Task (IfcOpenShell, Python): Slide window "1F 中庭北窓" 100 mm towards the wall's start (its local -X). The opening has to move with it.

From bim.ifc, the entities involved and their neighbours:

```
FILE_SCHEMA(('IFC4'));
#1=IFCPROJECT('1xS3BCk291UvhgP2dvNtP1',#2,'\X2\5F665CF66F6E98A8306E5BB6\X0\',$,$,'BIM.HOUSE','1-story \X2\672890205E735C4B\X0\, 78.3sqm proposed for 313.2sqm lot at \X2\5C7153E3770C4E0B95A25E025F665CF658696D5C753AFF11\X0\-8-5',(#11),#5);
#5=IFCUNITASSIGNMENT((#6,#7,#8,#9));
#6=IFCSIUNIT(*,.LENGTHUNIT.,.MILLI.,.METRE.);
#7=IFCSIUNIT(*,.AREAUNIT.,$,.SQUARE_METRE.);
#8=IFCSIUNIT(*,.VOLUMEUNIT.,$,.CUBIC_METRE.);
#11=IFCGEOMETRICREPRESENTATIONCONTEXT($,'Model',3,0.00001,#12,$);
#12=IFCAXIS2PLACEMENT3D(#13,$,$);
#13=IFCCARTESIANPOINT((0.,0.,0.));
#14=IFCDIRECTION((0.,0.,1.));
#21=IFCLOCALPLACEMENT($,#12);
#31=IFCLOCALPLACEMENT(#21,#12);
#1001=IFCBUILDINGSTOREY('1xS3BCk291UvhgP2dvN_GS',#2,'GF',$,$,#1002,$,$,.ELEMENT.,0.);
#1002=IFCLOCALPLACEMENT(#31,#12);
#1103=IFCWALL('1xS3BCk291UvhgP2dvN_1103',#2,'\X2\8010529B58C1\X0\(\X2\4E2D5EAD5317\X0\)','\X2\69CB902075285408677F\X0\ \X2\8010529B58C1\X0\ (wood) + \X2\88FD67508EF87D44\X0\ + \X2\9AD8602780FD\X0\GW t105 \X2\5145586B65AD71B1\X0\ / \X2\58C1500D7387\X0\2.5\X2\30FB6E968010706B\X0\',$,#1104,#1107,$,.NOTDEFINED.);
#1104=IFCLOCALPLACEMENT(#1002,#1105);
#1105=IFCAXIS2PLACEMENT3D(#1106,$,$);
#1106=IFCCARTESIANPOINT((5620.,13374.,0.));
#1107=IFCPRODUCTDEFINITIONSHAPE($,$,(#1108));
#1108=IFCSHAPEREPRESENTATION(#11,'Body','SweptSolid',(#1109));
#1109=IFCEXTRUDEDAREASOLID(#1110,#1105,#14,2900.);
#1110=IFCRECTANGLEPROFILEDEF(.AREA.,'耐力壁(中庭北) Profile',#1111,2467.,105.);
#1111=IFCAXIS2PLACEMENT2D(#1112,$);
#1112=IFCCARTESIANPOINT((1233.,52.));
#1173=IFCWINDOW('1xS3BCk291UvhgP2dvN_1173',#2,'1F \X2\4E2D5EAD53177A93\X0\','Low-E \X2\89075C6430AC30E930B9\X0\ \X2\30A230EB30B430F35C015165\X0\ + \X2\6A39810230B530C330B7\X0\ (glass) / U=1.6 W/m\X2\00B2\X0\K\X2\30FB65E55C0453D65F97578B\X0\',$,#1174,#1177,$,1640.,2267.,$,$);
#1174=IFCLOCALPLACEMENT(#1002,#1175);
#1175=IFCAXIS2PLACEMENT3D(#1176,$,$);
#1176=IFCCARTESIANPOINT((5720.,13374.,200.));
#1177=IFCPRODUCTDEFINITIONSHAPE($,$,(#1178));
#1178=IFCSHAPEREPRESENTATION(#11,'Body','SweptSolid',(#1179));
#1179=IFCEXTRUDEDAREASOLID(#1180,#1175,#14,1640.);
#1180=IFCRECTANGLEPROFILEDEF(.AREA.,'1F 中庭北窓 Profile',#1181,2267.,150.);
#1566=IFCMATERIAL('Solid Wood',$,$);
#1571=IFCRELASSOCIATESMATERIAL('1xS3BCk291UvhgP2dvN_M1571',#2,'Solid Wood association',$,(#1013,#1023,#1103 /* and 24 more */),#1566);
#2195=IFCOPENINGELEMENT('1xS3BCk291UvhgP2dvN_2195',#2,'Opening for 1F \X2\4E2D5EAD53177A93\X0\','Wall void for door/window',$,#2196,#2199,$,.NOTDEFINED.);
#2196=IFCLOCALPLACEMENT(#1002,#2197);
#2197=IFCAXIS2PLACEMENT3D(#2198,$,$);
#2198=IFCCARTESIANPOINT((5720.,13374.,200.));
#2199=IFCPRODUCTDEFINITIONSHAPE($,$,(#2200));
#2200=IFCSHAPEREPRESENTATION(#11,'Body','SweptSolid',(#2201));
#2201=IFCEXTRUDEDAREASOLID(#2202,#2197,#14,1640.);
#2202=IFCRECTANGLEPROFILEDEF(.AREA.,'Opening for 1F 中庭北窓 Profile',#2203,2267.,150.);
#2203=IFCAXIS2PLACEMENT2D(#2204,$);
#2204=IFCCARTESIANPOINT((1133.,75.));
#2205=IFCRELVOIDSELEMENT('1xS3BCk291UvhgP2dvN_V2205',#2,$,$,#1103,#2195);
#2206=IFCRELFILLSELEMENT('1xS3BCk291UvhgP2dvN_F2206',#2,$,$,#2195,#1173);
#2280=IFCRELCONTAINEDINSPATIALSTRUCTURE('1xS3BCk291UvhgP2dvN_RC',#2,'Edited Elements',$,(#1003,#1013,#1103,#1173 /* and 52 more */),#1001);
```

```python
import ifcopenshell
import ifcopenshell.api.geometry
import ifcopenshell.util.placement

model = ifcopenshell.open("bim.ifc")

window = model.by_guid("1xS3BCk291UvhgP2dvN_1173")
opening = window.FillsVoids[0].RelatingOpeningElement
wall = opening.VoidsElements[0].RelatingBuildingElement

wall_matrix = ifcopenshell.util.placement.get_local_placement(wall.ObjectPlacement)
shift = wall_matrix[:3, 0] * -100.0
before = ifcopenshell.util.placement.get_local_placement(window.ObjectPlacement)[:3, 3].copy()

# The window is not placed relative to its opening, so move both.
for product in (opening, window):
    matrix = ifcopenshell.util.placement.get_local_placement(product.ObjectPlacement)
    matrix[:3, 3] += shift
    ifcopenshell.api.geometry.edit_object_placement(model, product=product, matrix=matrix, is_si=False)

after = ifcopenshell.util.placement.get_local_placement(window.ObjectPlacement)[:3, 3]
print("window moved by", (after - before).round(3) + 0.0)

model.write("bim_v2.ifc")
```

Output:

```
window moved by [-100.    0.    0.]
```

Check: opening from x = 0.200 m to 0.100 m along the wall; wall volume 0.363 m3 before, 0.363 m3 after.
